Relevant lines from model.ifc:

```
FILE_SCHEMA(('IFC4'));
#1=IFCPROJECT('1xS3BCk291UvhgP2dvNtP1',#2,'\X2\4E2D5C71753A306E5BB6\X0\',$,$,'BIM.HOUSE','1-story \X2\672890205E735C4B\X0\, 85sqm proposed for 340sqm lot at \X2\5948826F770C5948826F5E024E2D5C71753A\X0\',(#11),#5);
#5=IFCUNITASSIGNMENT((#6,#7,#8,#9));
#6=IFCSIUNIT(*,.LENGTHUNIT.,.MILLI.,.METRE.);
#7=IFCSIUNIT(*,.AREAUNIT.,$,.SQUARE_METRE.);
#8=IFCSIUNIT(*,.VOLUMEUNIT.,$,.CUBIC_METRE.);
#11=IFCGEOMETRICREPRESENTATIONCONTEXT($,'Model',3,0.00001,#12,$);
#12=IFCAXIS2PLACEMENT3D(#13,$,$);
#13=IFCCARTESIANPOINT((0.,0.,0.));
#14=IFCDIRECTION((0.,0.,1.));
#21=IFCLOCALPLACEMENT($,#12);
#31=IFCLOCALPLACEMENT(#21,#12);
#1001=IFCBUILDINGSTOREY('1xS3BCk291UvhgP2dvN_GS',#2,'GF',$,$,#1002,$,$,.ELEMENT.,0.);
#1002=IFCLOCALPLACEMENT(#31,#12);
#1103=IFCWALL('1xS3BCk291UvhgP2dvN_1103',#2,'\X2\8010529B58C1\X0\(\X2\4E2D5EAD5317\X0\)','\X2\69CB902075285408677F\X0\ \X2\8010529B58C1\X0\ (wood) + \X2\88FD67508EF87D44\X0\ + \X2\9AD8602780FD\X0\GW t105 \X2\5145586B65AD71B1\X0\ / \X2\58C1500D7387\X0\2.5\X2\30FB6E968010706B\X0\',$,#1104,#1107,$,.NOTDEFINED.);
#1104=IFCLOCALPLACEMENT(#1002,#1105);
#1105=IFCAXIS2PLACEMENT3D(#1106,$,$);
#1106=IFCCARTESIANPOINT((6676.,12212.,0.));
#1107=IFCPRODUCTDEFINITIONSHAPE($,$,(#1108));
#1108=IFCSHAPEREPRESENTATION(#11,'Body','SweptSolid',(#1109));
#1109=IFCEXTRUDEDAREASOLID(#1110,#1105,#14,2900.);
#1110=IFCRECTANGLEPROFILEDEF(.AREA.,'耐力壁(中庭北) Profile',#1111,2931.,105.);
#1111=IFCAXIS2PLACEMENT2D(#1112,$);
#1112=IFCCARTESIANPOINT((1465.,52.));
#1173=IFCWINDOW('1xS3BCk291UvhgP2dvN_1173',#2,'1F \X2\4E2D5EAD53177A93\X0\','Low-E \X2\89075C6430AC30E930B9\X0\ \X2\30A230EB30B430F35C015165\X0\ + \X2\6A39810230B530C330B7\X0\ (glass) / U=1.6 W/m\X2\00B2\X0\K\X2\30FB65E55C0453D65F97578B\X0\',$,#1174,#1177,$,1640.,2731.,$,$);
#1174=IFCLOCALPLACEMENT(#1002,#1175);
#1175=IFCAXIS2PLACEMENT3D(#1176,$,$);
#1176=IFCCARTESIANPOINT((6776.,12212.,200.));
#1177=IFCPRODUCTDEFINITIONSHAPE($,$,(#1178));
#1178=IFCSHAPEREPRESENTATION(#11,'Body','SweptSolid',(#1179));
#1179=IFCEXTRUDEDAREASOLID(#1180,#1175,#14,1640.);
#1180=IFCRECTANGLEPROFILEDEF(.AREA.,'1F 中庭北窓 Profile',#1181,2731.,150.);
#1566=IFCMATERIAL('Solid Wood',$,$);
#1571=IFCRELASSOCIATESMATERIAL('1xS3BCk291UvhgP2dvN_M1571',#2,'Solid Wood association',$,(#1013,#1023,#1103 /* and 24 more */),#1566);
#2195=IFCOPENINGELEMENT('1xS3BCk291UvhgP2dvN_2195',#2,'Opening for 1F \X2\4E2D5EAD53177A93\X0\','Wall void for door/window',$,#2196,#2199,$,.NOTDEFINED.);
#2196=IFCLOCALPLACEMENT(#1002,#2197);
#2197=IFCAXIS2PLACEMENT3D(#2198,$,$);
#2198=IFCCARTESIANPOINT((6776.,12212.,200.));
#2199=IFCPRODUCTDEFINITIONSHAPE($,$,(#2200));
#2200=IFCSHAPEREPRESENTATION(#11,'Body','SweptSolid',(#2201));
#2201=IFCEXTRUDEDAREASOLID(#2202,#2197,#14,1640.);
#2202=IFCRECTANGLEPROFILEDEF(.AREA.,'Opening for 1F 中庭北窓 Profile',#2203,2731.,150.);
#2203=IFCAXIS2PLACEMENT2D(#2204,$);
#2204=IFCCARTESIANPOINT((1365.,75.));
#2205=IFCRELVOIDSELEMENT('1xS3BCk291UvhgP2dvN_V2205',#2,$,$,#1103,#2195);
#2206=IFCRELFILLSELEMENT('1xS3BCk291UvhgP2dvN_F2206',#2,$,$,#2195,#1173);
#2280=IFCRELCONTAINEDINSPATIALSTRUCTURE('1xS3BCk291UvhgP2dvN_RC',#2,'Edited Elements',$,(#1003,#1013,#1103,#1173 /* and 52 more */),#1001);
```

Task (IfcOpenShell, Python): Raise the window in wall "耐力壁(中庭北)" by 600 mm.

```python
import numpy as np
import ifcopenshell
import ifcopenshell.api.geometry
import ifcopenshell.util.placement
import ifcopenshell.util.unit

model = ifcopenshell.open("model.ifc")
unit_scale = ifcopenshell.util.unit.calculate_unit_scale(model)

window = model.by_id(1173)
opening = window.FillsVoids[0].RelatingOpeningElement
dz = 600.0

shift = np.array([0.0, 0.0, dz])
# The window is not placed relative to its opening, so move both.
for product in (opening, window):
    matrix = ifcopenshell.util.placement.get_local_placement(product.ObjectPlacement)
    matrix[:3, 3] += shift
    ifcopenshell.api.geometry.edit_object_placement(model, product=product, matrix=matrix, is_si=False)

print(f"moved by {dz * unit_scale:+.3f} m")

model.write("model_updated.ifc")
```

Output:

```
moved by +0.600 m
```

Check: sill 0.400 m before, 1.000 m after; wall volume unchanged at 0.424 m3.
